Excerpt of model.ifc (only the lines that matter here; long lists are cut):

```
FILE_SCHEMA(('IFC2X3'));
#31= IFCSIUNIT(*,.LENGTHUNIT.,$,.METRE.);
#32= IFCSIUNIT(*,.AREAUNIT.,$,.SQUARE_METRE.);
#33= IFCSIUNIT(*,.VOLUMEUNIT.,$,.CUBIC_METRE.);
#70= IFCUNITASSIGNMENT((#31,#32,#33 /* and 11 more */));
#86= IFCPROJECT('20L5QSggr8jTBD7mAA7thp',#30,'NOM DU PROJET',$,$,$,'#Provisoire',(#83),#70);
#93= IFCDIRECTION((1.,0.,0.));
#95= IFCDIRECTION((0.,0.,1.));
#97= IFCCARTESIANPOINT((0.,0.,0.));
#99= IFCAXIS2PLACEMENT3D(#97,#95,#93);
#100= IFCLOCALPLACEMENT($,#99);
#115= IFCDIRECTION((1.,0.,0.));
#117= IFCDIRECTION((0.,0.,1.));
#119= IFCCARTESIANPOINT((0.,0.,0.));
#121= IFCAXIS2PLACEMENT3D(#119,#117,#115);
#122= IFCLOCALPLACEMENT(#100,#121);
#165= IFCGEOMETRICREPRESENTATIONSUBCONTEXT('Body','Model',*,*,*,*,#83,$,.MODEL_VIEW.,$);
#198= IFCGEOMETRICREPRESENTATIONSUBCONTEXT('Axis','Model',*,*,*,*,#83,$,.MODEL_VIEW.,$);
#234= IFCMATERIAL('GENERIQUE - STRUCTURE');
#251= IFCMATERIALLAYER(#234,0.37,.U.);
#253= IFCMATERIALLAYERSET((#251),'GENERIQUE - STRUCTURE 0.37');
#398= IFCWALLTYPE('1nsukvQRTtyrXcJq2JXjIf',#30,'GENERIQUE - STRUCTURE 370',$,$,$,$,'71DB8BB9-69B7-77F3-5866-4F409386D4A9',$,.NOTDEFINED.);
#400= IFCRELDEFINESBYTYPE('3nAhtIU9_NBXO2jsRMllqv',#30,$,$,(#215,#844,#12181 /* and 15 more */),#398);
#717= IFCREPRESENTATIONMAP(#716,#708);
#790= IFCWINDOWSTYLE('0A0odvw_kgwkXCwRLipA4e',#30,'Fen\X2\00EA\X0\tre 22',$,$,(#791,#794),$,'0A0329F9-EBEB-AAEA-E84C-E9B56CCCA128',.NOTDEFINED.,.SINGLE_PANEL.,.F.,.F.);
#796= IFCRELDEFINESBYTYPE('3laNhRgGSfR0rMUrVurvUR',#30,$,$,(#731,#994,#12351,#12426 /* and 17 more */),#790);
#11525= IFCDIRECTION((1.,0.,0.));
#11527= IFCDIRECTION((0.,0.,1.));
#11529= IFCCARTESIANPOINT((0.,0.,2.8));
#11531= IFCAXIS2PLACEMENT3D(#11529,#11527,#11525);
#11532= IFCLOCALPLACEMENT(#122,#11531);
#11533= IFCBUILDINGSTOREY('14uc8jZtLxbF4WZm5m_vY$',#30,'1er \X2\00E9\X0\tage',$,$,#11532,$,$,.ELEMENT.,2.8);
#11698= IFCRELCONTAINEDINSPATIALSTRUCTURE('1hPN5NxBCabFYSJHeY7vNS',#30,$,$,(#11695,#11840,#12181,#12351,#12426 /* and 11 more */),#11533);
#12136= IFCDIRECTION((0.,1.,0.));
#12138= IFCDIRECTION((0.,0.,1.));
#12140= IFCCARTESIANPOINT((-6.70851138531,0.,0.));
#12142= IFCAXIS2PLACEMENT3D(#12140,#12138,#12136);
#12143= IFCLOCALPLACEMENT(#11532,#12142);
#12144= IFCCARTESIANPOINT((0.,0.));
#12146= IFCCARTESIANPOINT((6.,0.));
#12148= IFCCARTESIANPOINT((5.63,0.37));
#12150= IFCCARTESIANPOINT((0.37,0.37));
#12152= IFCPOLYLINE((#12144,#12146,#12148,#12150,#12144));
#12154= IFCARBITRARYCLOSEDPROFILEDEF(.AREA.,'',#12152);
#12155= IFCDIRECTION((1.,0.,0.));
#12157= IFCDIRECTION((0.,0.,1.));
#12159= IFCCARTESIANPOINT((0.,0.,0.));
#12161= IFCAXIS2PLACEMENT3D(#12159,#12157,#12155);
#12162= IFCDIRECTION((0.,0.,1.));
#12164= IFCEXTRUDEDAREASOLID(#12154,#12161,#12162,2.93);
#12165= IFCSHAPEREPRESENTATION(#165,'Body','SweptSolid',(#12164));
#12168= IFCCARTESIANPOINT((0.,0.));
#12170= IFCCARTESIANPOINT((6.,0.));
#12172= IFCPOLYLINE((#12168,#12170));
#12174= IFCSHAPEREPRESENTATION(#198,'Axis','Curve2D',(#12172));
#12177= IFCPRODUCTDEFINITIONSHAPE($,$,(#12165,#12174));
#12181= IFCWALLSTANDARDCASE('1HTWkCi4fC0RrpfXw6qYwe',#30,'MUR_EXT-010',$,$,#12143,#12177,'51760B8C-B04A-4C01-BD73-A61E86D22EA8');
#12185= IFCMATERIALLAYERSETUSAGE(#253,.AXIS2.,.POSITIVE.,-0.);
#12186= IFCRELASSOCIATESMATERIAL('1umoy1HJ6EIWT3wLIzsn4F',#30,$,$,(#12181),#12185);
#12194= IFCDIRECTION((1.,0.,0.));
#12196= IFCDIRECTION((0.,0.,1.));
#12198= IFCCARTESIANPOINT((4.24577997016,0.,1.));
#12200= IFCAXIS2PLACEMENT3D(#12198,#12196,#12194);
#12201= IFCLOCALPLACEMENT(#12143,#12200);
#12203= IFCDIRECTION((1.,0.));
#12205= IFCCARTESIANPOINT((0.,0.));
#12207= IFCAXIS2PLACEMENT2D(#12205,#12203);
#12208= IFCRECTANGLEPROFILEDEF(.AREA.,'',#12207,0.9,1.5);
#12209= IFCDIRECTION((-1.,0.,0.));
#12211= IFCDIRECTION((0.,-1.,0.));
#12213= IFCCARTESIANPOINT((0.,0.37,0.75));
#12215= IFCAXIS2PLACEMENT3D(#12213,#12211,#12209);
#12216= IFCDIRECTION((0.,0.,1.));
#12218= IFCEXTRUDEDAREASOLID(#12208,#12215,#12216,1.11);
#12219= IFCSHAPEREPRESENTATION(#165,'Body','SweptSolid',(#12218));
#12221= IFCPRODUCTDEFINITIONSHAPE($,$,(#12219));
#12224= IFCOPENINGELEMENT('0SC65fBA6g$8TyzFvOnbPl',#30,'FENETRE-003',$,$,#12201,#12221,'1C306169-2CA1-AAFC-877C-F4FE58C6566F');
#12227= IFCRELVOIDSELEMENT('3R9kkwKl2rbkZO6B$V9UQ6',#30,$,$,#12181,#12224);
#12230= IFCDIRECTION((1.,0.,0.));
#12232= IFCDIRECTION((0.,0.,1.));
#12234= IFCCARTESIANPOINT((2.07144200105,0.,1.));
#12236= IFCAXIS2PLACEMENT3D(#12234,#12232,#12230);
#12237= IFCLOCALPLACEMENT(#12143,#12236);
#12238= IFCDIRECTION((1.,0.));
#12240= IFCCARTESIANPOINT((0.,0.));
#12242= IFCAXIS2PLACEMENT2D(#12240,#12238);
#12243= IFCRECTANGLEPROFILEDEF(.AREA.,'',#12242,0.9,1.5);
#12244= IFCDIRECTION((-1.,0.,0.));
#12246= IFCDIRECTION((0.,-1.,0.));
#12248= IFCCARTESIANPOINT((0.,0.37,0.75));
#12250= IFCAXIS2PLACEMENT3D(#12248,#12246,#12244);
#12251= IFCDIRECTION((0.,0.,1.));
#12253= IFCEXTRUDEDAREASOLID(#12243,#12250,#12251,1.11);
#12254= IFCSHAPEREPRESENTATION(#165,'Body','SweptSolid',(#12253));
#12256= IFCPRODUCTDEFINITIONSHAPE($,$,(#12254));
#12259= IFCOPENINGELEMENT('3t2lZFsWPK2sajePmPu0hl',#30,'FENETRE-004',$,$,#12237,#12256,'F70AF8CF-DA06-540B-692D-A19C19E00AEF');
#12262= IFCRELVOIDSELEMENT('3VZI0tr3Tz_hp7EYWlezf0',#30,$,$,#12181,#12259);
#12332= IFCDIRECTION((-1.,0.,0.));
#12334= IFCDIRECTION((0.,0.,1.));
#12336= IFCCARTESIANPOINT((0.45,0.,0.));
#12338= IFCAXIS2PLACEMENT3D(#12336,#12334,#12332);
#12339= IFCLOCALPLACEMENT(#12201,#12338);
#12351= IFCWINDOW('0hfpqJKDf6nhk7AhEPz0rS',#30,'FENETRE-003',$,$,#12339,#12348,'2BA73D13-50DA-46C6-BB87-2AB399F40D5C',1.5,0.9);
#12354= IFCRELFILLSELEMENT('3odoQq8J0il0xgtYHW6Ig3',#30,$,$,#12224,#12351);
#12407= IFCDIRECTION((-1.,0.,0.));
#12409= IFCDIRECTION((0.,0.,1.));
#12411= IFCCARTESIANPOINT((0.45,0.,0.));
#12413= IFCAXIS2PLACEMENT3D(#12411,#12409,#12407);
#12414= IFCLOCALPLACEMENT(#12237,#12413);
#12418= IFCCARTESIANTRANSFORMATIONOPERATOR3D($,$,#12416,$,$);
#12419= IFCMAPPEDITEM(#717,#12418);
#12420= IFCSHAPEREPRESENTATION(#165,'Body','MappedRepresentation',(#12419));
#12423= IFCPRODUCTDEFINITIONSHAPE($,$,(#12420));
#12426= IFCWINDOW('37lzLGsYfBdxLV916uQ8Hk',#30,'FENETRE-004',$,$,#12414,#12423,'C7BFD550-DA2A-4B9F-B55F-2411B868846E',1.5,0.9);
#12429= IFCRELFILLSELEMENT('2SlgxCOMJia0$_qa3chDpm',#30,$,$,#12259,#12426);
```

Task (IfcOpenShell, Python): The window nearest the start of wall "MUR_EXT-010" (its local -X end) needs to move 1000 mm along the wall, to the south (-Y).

```python
import ifcopenshell
import ifcopenshell.api.geometry
import ifcopenshell.util.placement

model = ifcopenshell.open("model.ifc")

window = model.by_guid("37lzLGsYfBdxLV916uQ8Hk")
opening = window.FillsVoids[0].RelatingOpeningElement
wall = opening.VoidsElements[0].RelatingBuildingElement

wall_matrix = ifcopenshell.util.placement.get_local_placement(wall.ObjectPlacement)
shift = wall_matrix[:3, 0] * -1.0
before = ifcopenshell.util.placement.get_local_placement(window.ObjectPlacement)[:3, 3].copy()

# The window is placed relative to its opening, so it follows when the opening moves.
matrix = ifcopenshell.util.placement.get_local_placement(opening.ObjectPlacement)
matrix[:3, 3] += shift
ifcopenshell.api.geometry.edit_object_placement(
    model, product=opening, matrix=matrix, is_si=False, should_transform_children=True
)

after = ifcopenshell.util.placement.get_local_placement(window.ObjectPlacement)[:3, 3]
print("window moved by", (after - before).round(3) + 0.0)

model.write("model_rev.ifc")
```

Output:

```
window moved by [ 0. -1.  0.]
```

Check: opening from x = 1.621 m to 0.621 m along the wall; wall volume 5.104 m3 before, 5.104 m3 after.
